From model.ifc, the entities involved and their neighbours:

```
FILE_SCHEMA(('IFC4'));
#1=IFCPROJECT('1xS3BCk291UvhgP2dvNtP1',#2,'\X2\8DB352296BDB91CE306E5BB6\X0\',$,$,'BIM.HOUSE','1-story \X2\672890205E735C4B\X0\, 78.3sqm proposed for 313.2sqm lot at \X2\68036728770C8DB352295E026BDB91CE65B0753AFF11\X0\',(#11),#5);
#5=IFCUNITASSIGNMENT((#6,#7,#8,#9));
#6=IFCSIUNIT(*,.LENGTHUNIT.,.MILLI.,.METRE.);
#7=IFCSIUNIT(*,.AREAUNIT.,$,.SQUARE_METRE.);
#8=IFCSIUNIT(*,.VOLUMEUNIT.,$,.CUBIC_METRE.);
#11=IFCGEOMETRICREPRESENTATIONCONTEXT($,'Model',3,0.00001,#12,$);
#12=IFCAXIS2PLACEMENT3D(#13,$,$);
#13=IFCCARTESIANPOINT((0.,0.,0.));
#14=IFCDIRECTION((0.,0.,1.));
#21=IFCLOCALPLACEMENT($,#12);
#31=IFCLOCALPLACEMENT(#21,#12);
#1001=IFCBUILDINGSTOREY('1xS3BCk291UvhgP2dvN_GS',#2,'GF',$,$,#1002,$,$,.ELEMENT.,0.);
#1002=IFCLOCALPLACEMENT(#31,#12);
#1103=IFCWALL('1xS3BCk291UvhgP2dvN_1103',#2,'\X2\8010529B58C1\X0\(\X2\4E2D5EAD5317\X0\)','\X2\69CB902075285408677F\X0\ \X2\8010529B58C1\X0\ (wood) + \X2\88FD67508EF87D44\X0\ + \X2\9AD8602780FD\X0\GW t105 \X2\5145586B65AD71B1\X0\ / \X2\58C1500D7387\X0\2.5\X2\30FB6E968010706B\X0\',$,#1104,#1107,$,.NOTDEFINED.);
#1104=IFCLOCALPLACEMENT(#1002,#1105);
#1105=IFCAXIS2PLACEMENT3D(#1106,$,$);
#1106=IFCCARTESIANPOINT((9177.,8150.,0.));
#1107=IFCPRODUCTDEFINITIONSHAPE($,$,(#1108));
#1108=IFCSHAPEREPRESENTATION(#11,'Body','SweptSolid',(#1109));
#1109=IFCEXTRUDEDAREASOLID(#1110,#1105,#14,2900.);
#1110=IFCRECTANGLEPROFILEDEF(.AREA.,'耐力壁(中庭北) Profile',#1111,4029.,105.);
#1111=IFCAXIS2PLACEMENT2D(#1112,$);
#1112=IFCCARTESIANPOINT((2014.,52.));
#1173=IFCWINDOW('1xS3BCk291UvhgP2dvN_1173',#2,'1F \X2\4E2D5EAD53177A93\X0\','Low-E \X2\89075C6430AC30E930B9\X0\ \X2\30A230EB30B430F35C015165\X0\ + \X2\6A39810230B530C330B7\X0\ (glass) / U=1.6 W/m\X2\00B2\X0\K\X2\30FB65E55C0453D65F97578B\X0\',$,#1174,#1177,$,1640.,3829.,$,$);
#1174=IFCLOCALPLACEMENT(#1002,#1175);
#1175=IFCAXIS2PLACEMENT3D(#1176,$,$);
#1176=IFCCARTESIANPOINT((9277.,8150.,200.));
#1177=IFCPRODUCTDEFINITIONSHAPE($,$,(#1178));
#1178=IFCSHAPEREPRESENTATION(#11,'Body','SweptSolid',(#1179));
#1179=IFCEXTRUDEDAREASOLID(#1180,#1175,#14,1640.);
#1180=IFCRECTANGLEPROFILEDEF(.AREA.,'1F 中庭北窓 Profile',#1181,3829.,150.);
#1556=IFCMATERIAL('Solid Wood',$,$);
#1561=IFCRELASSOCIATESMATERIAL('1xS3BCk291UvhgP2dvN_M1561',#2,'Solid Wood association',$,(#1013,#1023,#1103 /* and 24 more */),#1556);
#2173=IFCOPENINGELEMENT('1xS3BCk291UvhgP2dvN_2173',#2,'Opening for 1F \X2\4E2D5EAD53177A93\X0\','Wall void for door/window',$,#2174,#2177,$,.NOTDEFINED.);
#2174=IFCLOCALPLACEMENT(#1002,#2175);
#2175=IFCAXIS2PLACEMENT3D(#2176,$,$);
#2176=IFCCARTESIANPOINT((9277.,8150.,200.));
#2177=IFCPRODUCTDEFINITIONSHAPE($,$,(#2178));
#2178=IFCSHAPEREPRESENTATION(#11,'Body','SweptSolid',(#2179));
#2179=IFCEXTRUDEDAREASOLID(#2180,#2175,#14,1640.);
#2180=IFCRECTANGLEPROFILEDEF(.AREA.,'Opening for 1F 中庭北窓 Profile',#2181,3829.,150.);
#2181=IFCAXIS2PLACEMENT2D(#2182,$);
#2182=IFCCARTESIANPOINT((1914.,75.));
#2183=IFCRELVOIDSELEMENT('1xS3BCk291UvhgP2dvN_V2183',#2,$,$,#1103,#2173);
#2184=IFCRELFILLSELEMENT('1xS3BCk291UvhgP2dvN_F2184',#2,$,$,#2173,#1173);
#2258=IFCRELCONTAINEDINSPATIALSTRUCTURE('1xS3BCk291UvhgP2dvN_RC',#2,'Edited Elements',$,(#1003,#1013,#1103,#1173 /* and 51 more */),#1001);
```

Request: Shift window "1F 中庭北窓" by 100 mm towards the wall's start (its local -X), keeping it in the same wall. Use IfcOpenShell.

```python
import ifcopenshell
import ifcopenshell.api.geometry
import ifcopenshell.util.placement

model = ifcopenshell.open("model.ifc")

window = model.by_id(1173)
opening = window.FillsVoids[0].RelatingOpeningElement
wall = opening.VoidsElements[0].RelatingBuildingElement

wall_matrix = ifcopenshell.util.placement.get_local_placement(wall.ObjectPlacement)
shift = wall_matrix[:3, 0] * -100.0
before = ifcopenshell.util.placement.get_local_placement(window.ObjectPlacement)[:3, 3].copy()

# The window is not placed relative to its opening, so move both.
for product in (opening, window):
    matrix = ifcopenshell.util.placement.get_local_placement(product.ObjectPlacement)
    matrix[:3, 3] += shift
    ifcopenshell.api.geometry.edit_object_placement(model, product=product, matrix=matrix, is_si=False)

after = ifcopenshell.util.placement.get_local_placement(window.ObjectPlacement)[:3, 3]
print("window moved by", (after - before).round(3) + 0.0)

model.write("model_rev.ifc")
```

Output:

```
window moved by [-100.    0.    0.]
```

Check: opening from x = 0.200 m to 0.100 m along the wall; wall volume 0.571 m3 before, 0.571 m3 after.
